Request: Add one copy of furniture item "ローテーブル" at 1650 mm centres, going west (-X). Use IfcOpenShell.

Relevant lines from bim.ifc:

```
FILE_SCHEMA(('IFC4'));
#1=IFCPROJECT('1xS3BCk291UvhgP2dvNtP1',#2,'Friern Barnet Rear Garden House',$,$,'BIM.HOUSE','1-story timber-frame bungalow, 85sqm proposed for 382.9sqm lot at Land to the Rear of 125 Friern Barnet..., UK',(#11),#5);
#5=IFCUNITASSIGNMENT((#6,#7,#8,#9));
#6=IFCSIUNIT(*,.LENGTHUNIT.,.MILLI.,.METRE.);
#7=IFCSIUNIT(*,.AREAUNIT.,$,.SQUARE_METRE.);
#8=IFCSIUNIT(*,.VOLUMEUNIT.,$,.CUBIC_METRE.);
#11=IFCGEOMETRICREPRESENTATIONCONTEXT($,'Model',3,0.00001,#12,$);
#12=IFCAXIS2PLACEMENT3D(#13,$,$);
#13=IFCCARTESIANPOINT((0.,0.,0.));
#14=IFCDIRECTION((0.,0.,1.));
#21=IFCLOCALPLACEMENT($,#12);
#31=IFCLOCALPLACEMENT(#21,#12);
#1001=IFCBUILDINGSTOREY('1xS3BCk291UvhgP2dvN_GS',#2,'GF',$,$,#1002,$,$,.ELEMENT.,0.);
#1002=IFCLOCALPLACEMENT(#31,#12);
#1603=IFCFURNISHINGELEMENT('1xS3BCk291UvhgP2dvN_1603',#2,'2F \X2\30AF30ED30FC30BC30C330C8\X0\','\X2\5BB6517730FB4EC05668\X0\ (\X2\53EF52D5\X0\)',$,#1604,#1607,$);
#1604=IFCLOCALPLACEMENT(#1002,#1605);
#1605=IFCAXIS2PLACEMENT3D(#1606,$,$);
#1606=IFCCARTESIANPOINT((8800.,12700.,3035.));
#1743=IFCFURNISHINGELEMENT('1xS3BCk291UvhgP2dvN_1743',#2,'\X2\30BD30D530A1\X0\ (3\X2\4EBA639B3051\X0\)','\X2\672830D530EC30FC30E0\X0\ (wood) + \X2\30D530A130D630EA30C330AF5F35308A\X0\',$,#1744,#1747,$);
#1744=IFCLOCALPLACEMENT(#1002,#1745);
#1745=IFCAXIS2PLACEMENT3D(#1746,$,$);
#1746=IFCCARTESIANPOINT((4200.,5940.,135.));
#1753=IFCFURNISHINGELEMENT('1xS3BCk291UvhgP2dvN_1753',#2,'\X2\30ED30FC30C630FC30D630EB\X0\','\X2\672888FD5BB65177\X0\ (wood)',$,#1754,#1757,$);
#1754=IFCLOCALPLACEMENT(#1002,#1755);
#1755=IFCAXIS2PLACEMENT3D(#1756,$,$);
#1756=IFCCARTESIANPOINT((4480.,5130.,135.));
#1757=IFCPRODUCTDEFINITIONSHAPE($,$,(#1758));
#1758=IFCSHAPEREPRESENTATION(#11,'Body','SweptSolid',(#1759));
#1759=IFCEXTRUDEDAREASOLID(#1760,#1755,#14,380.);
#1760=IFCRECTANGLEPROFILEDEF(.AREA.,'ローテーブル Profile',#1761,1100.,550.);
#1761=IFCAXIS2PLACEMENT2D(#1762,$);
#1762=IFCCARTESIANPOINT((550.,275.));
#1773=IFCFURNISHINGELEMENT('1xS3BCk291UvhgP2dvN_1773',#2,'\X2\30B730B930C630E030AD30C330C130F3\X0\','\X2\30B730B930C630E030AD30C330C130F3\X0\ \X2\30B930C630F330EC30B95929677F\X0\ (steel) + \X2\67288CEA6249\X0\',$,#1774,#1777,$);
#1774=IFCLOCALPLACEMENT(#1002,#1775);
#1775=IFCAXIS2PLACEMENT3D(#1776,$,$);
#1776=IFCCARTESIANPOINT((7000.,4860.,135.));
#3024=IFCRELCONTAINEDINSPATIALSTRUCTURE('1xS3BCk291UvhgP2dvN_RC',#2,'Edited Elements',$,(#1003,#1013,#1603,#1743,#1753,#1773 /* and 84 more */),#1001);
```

```python
import numpy as np
import ifcopenshell
import ifcopenshell.api.geometry
import ifcopenshell.api.root
import ifcopenshell.util.element
import ifcopenshell.util.placement

model = ifcopenshell.open("bim.ifc")


def reuse_history(source, copy):
    """copy_class also copies each property set's owner history, people and application; keep the originals."""
    for rel in copy.IsDefinedBy:
        if rel.is_a("IfcRelDefinesByProperties") and (history := rel.RelatingPropertyDefinition.OwnerHistory):
            rel.RelatingPropertyDefinition.OwnerHistory = source.OwnerHistory
            ifcopenshell.util.element.remove_deep2(model, history)


source = model.by_id(1753)
base = ifcopenshell.util.placement.get_local_placement(source.ObjectPlacement)
step = np.array([-1.0, 0.0, 0.0]) * 1650.0

for i in range(1, 2):
    copy = ifcopenshell.api.root.copy_class(model, product=source)
    copy.Representation = ifcopenshell.util.element.copy_deep(
        model, source.Representation, exclude=["IfcGeometricRepresentationContext", "IfcRepresentationMap"]
    )
    reuse_history(source, copy)
    matrix = base.copy()
    matrix[:3, 3] += i * step
    print("added at", matrix[:3, 3].round(3) + 0.0)
    ifcopenshell.api.geometry.edit_object_placement(model, product=copy, matrix=matrix, is_si=False)

model.write("bim_edited.ifc")
```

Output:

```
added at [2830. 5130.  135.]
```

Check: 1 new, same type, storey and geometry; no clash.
